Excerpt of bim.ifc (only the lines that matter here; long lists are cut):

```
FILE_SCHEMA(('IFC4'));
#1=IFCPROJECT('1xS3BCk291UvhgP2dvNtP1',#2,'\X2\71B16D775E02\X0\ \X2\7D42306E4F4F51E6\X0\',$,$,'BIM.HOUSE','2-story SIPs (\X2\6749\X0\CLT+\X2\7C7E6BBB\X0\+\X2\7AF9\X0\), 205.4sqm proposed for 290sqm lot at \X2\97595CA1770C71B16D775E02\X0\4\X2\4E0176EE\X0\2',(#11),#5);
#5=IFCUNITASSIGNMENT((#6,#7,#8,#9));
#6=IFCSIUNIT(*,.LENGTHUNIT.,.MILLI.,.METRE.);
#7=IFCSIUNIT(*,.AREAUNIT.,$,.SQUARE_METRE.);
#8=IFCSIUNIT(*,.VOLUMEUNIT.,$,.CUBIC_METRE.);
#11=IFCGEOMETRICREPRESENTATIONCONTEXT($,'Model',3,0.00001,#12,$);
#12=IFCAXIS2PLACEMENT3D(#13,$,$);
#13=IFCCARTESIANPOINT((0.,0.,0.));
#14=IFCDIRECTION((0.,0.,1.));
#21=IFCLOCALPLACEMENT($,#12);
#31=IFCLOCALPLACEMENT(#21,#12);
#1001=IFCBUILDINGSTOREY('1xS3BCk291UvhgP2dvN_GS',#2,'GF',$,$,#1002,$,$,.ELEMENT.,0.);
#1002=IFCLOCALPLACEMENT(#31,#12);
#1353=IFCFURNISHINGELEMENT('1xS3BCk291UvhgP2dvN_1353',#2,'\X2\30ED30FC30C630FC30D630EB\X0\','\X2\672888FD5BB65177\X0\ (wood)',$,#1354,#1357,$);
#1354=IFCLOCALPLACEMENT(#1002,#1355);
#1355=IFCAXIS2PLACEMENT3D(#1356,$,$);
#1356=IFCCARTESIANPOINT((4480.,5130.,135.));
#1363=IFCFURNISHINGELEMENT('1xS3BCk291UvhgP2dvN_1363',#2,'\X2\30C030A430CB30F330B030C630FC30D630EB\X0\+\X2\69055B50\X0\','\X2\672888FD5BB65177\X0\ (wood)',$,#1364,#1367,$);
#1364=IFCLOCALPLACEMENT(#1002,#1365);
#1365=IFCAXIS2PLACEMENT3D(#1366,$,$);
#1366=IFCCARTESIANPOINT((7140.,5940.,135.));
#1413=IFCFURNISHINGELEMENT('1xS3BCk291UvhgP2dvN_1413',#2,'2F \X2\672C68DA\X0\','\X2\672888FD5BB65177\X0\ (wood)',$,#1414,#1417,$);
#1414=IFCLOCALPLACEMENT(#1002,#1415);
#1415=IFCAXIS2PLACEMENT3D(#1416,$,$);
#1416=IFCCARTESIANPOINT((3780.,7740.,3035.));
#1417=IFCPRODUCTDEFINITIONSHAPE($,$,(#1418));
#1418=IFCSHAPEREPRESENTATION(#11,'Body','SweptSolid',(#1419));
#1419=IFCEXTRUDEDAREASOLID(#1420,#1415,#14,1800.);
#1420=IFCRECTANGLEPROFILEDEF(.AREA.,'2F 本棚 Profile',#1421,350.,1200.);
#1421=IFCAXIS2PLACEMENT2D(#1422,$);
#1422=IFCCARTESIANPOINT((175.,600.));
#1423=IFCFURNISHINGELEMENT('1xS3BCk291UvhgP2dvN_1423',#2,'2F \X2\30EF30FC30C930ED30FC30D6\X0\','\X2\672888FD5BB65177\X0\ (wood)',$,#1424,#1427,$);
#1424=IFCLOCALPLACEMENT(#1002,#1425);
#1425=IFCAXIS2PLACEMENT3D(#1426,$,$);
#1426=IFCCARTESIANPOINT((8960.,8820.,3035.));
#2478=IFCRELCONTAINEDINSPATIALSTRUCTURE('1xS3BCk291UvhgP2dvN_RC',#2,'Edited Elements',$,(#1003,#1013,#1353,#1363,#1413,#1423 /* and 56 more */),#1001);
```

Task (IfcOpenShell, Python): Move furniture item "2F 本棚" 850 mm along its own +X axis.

```python
import ifcopenshell
import ifcopenshell.api.geometry
import ifcopenshell.util.placement

model = ifcopenshell.open("bim.ifc")

item = model.by_guid("1xS3BCk291UvhgP2dvN_1413")
matrix = ifcopenshell.util.placement.get_local_placement(item.ObjectPlacement)
matrix[:3, 3] += matrix[:3, 0] * 850.0
ifcopenshell.api.geometry.edit_object_placement(model, product=item, matrix=matrix, is_si=False)

print(ifcopenshell.util.placement.get_local_placement(item.ObjectPlacement).round(3) + 0.0)

model.write("bim_rev.ifc")
```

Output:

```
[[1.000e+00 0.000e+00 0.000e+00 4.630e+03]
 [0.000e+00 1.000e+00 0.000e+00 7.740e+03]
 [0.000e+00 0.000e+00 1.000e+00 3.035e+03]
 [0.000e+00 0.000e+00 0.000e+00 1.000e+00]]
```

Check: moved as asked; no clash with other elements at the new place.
